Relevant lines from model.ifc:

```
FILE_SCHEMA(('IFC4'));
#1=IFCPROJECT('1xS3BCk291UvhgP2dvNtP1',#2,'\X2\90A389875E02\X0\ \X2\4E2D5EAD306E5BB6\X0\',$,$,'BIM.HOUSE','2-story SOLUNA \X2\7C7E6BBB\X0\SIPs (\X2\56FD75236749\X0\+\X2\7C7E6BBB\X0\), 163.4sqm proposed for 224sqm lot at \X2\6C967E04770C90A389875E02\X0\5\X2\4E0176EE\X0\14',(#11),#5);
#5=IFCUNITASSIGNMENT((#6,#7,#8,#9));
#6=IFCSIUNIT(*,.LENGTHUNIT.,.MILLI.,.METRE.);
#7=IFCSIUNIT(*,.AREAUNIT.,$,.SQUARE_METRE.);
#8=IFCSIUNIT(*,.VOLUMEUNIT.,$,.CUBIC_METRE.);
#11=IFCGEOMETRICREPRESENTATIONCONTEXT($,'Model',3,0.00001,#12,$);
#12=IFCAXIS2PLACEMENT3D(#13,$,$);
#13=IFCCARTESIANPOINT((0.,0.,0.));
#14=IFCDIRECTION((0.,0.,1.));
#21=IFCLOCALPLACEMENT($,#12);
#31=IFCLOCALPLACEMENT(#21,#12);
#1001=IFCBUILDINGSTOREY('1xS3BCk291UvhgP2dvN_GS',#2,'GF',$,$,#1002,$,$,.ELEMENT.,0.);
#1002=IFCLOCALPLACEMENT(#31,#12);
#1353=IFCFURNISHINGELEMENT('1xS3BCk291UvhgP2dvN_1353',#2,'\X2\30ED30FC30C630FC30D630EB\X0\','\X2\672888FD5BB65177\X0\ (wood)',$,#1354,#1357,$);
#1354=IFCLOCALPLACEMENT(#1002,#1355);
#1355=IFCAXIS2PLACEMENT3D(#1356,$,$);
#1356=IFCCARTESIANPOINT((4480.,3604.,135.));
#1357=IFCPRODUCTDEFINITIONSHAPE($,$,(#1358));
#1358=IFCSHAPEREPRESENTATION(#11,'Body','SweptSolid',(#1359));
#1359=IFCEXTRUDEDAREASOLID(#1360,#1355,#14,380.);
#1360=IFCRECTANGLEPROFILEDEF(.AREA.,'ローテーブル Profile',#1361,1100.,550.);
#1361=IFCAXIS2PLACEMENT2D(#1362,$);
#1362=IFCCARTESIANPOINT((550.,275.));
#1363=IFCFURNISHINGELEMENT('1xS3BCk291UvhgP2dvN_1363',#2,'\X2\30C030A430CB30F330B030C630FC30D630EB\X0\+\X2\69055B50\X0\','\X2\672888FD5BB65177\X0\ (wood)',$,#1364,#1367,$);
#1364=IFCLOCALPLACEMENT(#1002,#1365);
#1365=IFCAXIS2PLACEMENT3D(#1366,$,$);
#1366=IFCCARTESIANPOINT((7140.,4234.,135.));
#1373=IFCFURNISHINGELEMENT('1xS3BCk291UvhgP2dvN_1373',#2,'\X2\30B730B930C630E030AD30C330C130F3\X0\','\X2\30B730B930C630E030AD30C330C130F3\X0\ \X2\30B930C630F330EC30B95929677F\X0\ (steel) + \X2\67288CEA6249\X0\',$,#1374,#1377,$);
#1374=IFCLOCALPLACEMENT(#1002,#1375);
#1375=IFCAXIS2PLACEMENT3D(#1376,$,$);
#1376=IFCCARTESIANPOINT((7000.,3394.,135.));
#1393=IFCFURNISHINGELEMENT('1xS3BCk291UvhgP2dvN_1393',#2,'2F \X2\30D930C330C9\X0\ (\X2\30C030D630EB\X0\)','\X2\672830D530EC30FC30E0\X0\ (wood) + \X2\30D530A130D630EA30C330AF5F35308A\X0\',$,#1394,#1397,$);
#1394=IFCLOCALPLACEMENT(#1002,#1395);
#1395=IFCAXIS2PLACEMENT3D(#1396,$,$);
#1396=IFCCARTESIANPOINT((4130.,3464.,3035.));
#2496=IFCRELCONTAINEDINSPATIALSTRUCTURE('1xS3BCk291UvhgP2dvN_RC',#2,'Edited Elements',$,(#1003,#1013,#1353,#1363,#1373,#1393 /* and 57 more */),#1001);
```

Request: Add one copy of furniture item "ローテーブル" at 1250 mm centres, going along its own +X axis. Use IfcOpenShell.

```python
import ifcopenshell
import ifcopenshell.api.geometry
import ifcopenshell.api.root
import ifcopenshell.util.element
import ifcopenshell.util.placement

model = ifcopenshell.open("model.ifc")


def reuse_history(source, copy):
    """copy_class also copies each property set's owner history, people and application; keep the originals."""
    for rel in copy.IsDefinedBy:
        if rel.is_a("IfcRelDefinesByProperties") and (history := rel.RelatingPropertyDefinition.OwnerHistory):
            rel.RelatingPropertyDefinition.OwnerHistory = source.OwnerHistory
            ifcopenshell.util.element.remove_deep2(model, history)


source = model.by_guid("1xS3BCk291UvhgP2dvN_1353")
base = ifcopenshell.util.placement.get_local_placement(source.ObjectPlacement)
step = base[:3, 0] * 1250.0

for i in range(1, 2):
    copy = ifcopenshell.api.root.copy_class(model, product=source)
    copy.Representation = ifcopenshell.util.element.copy_deep(
        model, source.Representation, exclude=["IfcGeometricRepresentationContext", "IfcRepresentationMap"]
    )
    reuse_history(source, copy)
    matrix = base.copy()
    matrix[:3, 3] += i * step
    print("added at", matrix[:3, 3].round(3) + 0.0)
    ifcopenshell.api.geometry.edit_object_placement(model, product=copy, matrix=matrix, is_si=False)

model.write("model-out.ifc")
```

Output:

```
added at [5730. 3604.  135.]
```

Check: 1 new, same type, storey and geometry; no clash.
